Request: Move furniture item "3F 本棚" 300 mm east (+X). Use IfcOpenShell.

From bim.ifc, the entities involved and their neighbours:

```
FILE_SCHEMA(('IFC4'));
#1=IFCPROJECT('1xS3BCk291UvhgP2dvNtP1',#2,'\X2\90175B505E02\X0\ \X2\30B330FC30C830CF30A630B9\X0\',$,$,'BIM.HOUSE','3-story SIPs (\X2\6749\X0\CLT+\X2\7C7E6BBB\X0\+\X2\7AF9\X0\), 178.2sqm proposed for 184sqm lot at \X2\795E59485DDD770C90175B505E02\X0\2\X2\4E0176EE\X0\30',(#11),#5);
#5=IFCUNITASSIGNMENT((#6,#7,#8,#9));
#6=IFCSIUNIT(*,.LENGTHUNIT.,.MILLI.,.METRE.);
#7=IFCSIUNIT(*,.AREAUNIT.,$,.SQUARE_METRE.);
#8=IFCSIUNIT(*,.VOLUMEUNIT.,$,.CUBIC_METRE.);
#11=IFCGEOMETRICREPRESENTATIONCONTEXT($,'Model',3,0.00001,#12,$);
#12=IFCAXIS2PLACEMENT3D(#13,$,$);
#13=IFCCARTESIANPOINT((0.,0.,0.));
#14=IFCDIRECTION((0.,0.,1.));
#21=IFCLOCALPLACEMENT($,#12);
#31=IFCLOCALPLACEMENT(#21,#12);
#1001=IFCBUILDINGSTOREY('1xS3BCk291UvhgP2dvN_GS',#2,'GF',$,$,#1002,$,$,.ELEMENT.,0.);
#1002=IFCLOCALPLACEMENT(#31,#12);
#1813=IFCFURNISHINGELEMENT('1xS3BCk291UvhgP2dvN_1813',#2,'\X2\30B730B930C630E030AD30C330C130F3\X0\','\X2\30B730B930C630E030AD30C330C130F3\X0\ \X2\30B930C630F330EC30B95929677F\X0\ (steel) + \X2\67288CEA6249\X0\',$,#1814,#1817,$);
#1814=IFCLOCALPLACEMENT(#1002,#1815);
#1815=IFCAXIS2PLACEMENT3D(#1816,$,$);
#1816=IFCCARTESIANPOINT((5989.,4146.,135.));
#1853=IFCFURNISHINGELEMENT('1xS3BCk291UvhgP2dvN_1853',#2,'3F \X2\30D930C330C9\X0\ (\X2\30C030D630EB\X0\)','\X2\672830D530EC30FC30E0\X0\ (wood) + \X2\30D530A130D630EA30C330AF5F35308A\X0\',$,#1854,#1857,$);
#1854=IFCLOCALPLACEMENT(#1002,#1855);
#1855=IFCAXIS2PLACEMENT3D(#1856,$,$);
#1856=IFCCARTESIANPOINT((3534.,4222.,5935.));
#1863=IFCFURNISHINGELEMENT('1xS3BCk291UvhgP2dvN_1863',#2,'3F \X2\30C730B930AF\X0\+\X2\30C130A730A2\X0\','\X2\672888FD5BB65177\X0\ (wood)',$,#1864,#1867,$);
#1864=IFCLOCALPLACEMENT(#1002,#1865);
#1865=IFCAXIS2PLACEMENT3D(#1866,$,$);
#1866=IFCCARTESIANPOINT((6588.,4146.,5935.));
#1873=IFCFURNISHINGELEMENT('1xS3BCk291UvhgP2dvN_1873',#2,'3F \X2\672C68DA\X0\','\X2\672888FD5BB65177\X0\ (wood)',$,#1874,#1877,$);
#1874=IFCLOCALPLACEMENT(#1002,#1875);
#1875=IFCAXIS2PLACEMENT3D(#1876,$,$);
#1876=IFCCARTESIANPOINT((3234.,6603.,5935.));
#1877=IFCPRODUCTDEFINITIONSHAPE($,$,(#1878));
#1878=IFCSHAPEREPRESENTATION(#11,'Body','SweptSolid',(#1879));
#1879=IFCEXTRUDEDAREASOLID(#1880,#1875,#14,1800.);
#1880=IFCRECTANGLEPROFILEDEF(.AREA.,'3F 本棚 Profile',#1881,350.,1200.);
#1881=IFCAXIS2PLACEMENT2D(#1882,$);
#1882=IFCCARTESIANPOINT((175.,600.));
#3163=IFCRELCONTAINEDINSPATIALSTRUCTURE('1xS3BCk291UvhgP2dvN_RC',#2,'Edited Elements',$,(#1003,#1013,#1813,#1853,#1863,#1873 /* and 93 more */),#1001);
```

```python
import ifcopenshell
import ifcopenshell.api.geometry
import ifcopenshell.util.placement
import ifcopenshell.util.unit

model = ifcopenshell.open("bim.ifc")
unit_scale = ifcopenshell.util.unit.calculate_unit_scale(model)

item = model.by_guid("1xS3BCk291UvhgP2dvN_1873")
matrix = ifcopenshell.util.placement.get_local_placement(item.ObjectPlacement)
matrix[0, 3] += 0.3 / unit_scale
ifcopenshell.api.geometry.edit_object_placement(model, product=item, matrix=matrix, is_si=False)

print(ifcopenshell.util.placement.get_local_placement(item.ObjectPlacement).round(3) + 0.0)

model.write("bim_rev.ifc")
```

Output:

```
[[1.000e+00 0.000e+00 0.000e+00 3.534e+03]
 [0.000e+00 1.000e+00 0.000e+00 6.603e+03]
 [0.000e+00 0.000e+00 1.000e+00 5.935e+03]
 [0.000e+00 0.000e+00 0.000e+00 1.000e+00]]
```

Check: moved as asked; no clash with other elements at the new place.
